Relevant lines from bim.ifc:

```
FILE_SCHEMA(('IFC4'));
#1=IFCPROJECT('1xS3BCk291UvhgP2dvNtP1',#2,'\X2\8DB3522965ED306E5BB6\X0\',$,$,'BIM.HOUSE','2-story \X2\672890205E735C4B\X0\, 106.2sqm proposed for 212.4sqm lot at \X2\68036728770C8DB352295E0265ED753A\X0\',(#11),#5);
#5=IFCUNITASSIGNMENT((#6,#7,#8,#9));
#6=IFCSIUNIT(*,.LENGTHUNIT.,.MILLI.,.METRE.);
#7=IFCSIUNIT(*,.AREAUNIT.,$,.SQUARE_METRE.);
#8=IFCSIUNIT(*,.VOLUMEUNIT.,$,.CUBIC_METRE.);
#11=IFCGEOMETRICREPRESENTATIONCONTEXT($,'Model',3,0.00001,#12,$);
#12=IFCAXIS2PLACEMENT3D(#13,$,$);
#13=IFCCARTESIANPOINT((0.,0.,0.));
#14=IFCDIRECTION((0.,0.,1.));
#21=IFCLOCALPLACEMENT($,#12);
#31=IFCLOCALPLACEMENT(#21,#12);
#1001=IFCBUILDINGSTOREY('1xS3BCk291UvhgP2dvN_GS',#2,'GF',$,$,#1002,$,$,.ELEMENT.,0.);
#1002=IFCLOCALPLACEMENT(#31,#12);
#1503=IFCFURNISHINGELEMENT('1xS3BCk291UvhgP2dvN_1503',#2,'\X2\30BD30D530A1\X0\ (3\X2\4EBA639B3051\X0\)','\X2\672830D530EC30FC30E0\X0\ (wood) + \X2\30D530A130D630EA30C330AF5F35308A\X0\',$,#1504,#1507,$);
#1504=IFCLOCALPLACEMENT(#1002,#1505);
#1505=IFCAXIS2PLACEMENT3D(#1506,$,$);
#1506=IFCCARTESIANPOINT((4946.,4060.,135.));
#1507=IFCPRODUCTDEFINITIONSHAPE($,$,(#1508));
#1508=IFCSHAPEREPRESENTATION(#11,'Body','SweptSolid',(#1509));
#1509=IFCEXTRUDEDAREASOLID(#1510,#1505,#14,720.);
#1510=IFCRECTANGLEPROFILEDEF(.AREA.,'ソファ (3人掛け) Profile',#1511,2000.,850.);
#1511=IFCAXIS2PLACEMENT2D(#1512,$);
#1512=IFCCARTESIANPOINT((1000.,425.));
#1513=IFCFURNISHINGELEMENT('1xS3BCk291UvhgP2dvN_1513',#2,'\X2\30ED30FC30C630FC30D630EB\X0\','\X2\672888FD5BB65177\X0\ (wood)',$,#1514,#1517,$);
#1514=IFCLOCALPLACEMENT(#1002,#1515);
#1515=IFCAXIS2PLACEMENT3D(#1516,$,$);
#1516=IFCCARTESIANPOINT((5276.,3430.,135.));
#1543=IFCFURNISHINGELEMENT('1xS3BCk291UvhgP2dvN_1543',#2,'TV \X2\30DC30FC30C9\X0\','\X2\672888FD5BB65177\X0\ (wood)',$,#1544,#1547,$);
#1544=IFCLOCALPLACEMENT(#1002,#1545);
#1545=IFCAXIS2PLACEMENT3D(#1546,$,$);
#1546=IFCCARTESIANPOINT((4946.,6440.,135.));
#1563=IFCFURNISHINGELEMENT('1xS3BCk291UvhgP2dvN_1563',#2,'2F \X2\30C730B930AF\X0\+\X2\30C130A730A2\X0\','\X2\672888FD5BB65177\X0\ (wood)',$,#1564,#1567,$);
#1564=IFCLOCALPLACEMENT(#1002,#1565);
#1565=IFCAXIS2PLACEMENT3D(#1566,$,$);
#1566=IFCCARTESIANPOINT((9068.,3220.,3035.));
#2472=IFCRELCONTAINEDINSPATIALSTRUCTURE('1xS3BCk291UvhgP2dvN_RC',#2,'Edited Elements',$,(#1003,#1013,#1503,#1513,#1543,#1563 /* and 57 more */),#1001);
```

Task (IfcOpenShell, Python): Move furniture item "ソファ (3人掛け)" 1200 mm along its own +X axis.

```python
import ifcopenshell
import ifcopenshell.api.geometry
import ifcopenshell.util.placement

model = ifcopenshell.open("bim.ifc")

item = model.by_guid("1xS3BCk291UvhgP2dvN_1503")
matrix = ifcopenshell.util.placement.get_local_placement(item.ObjectPlacement)
matrix[:3, 3] += matrix[:3, 0] * 1200.0
ifcopenshell.api.geometry.edit_object_placement(model, product=item, matrix=matrix, is_si=False)

print(ifcopenshell.util.placement.get_local_placement(item.ObjectPlacement).round(3) + 0.0)

model.write("bim_rev.ifc")
```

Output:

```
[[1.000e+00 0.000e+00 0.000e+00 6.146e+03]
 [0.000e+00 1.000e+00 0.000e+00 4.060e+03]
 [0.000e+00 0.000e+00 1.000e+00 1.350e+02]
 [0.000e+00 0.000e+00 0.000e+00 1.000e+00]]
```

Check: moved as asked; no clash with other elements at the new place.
